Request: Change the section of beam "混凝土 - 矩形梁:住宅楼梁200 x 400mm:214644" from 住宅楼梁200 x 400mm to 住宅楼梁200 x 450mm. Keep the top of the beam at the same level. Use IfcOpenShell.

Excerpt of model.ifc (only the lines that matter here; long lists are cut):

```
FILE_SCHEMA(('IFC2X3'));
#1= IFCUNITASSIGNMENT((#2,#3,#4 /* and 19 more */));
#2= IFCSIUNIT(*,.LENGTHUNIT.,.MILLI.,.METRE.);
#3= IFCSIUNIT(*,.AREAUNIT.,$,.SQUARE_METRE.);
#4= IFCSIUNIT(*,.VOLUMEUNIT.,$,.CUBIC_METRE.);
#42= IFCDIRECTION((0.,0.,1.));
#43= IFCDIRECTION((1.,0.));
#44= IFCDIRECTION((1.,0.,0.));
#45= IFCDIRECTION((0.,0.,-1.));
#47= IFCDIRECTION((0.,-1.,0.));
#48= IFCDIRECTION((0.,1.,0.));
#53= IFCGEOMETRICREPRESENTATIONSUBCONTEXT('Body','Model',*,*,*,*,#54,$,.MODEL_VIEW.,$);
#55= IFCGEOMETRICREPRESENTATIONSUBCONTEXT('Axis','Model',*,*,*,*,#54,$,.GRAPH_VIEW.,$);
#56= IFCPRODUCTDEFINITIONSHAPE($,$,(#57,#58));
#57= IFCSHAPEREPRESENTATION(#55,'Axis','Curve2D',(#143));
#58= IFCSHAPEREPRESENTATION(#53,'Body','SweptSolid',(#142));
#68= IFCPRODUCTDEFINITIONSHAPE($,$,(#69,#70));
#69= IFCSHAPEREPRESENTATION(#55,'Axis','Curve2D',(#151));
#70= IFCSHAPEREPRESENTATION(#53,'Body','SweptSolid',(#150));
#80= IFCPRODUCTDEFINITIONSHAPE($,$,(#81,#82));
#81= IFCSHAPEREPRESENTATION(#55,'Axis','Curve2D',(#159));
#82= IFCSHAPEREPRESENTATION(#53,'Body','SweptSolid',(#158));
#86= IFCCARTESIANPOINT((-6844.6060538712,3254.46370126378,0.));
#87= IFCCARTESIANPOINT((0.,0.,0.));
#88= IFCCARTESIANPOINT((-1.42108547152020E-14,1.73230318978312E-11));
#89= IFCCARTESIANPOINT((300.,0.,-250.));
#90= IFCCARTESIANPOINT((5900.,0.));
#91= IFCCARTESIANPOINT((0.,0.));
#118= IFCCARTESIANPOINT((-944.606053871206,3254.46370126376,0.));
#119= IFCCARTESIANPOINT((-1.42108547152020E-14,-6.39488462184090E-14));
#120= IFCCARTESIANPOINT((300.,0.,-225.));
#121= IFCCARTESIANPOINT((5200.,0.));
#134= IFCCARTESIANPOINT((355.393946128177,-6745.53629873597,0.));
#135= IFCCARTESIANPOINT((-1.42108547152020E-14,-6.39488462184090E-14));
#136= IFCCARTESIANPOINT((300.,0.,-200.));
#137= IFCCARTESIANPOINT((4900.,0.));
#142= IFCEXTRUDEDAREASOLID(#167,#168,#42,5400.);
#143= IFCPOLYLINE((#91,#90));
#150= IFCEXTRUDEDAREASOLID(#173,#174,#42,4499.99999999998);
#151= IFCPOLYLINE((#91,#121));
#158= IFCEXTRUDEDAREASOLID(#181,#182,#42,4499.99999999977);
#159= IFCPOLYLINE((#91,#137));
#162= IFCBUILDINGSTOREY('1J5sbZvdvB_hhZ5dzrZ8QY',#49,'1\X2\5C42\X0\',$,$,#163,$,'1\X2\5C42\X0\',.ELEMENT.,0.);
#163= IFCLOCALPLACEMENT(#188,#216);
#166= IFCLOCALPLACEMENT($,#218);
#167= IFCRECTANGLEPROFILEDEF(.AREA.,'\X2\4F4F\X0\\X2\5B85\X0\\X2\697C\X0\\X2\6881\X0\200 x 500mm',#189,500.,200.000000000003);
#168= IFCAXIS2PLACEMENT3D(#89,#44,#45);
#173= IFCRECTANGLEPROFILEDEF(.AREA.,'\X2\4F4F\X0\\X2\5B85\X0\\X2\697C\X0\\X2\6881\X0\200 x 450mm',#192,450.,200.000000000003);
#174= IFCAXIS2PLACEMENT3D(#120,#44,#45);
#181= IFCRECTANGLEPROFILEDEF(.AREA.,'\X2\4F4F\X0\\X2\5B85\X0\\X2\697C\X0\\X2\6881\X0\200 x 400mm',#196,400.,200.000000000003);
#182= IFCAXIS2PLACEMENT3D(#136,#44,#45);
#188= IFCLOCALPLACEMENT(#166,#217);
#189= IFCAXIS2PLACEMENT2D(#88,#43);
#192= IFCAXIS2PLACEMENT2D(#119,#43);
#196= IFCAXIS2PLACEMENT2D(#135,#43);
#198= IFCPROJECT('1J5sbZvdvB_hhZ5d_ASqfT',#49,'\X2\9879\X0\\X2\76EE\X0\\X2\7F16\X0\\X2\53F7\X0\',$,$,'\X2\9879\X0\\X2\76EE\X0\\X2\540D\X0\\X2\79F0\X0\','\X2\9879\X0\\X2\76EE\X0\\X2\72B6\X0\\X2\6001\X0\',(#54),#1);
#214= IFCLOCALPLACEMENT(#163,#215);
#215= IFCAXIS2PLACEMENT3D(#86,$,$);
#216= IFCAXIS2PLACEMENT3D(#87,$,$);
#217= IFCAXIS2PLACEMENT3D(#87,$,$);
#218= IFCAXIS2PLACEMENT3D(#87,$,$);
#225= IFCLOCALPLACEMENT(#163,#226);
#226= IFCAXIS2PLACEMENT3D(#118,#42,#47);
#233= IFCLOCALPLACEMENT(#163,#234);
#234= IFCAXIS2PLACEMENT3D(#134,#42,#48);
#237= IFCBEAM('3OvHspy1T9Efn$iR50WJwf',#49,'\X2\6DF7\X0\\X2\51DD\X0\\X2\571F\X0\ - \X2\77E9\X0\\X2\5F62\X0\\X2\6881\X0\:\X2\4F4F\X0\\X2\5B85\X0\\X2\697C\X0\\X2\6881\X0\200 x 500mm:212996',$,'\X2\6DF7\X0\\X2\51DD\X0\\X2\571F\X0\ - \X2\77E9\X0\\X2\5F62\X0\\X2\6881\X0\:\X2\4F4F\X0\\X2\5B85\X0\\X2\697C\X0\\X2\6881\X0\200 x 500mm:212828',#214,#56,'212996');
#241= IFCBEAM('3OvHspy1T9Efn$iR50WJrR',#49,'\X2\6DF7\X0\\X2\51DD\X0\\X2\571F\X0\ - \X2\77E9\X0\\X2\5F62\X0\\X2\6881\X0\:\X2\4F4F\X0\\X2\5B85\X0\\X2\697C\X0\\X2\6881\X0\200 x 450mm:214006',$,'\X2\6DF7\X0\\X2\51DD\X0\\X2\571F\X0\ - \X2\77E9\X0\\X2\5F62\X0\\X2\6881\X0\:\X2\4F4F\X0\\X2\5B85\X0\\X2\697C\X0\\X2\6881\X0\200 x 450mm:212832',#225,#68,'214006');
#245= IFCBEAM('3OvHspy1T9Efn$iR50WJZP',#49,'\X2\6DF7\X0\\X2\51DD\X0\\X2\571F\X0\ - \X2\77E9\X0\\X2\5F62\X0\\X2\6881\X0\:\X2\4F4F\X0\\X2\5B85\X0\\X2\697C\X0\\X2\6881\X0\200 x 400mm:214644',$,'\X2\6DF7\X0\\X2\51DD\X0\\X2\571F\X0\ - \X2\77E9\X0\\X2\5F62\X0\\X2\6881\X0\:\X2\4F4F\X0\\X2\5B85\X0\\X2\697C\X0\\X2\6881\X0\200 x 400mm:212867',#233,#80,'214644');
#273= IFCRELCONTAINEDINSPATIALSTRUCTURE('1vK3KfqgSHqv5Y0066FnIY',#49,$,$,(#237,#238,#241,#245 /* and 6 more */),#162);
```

```python
import ifcopenshell
import ifcopenshell.util.element
import ifcopenshell.util.representation

model = ifcopenshell.open("model.ifc")

member = model.by_id(245)
source = next(p for p in model.by_type("IfcRectangleProfileDef") if p.ProfileName == "住宅楼梁200 x 450mm")

body = ifcopenshell.util.representation.get_representation(member, "Model", "Body")
solid = body.Items[0]
old_profile = solid.SweptArea

# Copy the section's sizes but keep this member's own profile position.
profile = ifcopenshell.util.element.copy(model, source)
# Profiles are centred, so shift by half the change in depth to hold the top.
shift = (old_profile.XDim - profile.XDim) / 2
x, y = old_profile.Position.Location.Coordinates
up = (-1.0, 0.0)  # upwards, in the solid's own plane
location = model.createIfcCartesianPoint((x + up[0] * shift, y + up[1] * shift))
profile.Position = model.createIfcAxis2Placement2D(location, old_profile.Position.RefDirection)
solid.SweptArea = profile
if not model.get_total_inverses(old_profile):
    ifcopenshell.util.element.remove_deep2(model, old_profile)
member.Name = member.Name.replace("住宅楼梁200 x 400mm", "住宅楼梁200 x 450mm")
member.ObjectType = member.ObjectType.replace("住宅楼梁200 x 400mm", "住宅楼梁200 x 450mm")

print(solid.SweptArea)

model.write("model_rev.ifc")
```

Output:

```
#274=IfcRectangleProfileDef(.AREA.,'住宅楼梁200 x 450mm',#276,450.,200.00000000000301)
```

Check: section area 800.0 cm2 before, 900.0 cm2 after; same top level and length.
